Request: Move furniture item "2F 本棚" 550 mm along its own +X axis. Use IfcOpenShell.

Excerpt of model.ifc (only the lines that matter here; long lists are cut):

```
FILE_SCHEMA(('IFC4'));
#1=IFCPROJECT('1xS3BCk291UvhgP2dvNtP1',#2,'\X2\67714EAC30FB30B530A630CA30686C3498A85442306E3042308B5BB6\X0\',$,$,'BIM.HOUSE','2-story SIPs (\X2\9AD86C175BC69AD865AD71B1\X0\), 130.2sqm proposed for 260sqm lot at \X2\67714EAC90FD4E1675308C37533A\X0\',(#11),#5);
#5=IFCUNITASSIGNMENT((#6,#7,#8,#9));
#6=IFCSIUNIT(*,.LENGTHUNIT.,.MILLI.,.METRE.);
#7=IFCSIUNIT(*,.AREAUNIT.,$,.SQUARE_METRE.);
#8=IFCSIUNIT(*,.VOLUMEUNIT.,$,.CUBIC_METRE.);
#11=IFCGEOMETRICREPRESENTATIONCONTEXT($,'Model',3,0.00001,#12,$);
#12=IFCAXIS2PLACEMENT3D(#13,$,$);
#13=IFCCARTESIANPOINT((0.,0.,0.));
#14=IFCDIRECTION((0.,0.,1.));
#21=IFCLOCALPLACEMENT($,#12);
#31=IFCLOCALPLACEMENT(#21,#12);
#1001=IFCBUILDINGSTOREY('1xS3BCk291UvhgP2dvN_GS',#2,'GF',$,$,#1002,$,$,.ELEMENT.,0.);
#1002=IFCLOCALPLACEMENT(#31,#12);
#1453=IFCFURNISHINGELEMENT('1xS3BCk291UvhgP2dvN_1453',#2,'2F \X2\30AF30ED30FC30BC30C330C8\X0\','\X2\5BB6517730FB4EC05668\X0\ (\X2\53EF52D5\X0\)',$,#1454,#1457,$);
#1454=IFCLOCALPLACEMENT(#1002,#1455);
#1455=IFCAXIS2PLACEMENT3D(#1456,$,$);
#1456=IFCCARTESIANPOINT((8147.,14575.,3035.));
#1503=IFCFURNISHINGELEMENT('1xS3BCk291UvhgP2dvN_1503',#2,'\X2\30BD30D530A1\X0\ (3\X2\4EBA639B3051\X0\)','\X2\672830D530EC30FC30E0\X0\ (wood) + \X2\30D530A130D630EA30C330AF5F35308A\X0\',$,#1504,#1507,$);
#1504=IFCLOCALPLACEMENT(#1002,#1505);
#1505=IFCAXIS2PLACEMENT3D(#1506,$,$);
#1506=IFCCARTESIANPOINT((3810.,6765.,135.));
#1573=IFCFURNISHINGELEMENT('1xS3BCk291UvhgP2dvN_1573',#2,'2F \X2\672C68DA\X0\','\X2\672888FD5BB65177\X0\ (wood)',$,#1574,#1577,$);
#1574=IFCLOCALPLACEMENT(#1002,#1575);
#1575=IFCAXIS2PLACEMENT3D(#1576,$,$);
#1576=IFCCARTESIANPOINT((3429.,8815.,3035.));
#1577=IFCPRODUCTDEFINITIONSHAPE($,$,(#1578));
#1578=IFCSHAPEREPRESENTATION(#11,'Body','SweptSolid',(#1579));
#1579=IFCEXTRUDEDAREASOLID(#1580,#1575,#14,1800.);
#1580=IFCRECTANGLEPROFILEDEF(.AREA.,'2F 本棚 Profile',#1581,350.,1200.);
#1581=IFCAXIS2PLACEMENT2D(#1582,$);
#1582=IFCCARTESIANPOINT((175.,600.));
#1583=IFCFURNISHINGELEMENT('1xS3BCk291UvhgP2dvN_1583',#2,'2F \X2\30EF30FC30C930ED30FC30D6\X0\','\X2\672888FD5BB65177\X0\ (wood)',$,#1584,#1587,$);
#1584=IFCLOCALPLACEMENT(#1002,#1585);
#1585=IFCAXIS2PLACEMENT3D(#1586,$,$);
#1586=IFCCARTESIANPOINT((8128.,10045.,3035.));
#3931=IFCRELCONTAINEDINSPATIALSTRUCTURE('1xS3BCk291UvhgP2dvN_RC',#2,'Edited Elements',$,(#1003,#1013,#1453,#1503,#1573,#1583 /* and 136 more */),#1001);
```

```python
import ifcopenshell
import ifcopenshell.api.geometry
import ifcopenshell.util.placement
import ifcopenshell.util.unit

model = ifcopenshell.open("model.ifc")
unit_scale = ifcopenshell.util.unit.calculate_unit_scale(model)

item = model.by_guid("1xS3BCk291UvhgP2dvN_1573")
matrix = ifcopenshell.util.placement.get_local_placement(item.ObjectPlacement)
matrix[:3, 3] += matrix[:3, 0] * 0.55 / unit_scale
ifcopenshell.api.geometry.edit_object_placement(model, product=item, matrix=matrix, is_si=False)

print(ifcopenshell.util.placement.get_local_placement(item.ObjectPlacement).round(3) + 0.0)

model.write("model_updated.ifc")
```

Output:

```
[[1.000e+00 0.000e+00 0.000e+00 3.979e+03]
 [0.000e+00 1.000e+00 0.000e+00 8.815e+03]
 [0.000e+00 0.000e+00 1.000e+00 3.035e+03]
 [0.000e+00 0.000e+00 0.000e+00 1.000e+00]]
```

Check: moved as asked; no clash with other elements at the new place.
